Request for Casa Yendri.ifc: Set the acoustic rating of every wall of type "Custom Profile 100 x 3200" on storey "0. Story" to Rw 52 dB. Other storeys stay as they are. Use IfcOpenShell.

First a look at what the model holds.

```python
import ifcopenshell
import ifcopenshell.util.element

model = ifcopenshell.open("Casa Yendri.ifc")
print(model.schema)
storey = next(s for s in model.by_type("IfcBuildingStorey") if s.Name == "0. Story")
walls = [e for e in ifcopenshell.util.element.get_decomposition(storey) if e.is_a("IfcWall")]
seen = {}
for e in walls:
    element_type = ifcopenshell.util.element.get_type(e)
    key = (element_type.Name if element_type != e and element_type else None, ifcopenshell.util.element.get_pset(e, "Pset_WallCommon", "AcousticRating"))
    seen[key] = seen.get(key, 0) + 1
for (name, value), count in sorted(seen.items(), key=str):
    print(count, "x", name, "|", value)
```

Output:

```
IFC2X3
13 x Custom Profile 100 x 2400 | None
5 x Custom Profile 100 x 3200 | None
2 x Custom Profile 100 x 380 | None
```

```python
import ifcopenshell
import ifcopenshell.api.pset
import ifcopenshell.util.element

model = ifcopenshell.open("Casa Yendri.ifc")

storey = next(s for s in model.by_type("IfcBuildingStorey") if s.Name == "0. Story")
walls = [e for e in ifcopenshell.util.element.get_decomposition(storey) if e.is_a("IfcWall")]

count = 0
for e in walls:
    element_type = ifcopenshell.util.element.get_type(e)
    if element_type in (None, e) or element_type.Name != "Custom Profile 100 x 3200":
        continue
    # add_pset returns the element's existing set when there is one.
    pset = ifcopenshell.api.pset.add_pset(model, product=e, name="Pset_WallCommon")
    ifcopenshell.api.pset.edit_pset(model, pset=pset, properties={"AcousticRating": "Rw 52 dB"})
    count += 1

print(count, "walls updated")

model.write("Casa Yendri_updated.ifc")
```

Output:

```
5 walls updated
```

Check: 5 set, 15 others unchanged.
